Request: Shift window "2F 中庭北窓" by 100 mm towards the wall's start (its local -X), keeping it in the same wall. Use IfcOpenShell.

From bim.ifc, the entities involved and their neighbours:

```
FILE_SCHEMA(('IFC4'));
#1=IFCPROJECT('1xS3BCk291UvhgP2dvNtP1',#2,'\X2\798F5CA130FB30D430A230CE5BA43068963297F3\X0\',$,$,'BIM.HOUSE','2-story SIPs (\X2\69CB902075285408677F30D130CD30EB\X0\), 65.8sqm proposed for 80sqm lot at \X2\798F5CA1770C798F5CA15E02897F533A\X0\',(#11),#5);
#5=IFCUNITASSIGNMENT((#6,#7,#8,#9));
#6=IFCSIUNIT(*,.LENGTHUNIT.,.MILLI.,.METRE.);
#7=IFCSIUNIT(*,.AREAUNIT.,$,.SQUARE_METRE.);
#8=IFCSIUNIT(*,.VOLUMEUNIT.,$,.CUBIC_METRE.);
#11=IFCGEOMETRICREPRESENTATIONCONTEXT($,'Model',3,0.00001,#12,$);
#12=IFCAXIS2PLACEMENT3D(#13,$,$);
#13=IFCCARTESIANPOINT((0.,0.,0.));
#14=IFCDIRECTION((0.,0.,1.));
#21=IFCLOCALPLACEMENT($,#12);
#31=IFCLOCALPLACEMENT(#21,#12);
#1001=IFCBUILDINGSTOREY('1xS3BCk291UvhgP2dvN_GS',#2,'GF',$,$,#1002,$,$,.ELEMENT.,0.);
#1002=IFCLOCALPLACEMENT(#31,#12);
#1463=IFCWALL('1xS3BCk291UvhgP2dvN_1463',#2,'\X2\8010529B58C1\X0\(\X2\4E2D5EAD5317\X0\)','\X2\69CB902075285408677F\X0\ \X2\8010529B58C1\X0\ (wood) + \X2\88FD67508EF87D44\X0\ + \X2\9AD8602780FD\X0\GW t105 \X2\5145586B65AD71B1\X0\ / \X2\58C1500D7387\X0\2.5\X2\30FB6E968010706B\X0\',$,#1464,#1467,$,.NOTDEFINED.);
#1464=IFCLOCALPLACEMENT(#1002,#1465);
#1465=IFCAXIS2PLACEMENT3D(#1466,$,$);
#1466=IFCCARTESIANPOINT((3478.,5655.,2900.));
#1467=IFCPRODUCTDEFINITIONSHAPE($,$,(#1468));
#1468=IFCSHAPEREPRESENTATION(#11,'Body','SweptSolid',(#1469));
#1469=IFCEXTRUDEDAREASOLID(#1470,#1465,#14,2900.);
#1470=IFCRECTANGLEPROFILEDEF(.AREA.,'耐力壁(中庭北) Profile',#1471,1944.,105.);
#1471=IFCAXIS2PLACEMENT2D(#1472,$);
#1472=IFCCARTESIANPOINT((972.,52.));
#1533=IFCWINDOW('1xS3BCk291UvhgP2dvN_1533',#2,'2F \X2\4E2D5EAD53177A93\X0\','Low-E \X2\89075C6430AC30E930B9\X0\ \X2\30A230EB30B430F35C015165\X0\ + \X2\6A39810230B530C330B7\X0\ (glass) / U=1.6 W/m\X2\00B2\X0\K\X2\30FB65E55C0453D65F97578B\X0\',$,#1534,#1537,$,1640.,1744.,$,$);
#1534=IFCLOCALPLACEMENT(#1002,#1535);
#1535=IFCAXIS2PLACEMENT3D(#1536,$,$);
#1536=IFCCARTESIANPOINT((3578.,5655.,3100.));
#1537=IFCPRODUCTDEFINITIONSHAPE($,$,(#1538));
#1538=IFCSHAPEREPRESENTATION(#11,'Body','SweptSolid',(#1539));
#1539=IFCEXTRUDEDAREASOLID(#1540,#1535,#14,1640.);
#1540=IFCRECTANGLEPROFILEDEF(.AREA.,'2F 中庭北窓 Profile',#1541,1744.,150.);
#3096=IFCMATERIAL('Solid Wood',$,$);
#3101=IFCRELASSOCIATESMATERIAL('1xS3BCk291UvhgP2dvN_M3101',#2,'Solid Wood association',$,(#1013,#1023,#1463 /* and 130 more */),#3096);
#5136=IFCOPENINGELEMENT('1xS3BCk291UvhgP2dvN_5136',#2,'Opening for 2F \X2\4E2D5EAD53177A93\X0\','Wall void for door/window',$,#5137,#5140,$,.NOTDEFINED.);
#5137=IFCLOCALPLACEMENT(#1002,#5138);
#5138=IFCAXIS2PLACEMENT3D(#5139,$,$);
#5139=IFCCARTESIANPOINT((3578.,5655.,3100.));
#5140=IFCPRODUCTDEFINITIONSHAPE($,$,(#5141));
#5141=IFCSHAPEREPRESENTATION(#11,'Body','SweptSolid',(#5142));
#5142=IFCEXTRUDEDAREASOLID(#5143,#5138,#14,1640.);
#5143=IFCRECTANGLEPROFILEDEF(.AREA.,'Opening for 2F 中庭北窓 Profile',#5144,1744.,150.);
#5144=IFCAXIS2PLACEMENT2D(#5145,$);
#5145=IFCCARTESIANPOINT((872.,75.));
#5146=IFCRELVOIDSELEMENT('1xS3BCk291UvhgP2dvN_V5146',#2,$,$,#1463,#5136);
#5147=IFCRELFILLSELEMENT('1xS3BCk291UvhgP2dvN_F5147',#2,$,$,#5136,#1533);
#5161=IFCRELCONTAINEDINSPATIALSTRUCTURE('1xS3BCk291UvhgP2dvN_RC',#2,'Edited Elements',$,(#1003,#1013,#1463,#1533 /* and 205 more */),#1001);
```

```python
import ifcopenshell
import ifcopenshell.api.geometry
import ifcopenshell.util.placement
import ifcopenshell.util.unit

model = ifcopenshell.open("bim.ifc")
unit_scale = ifcopenshell.util.unit.calculate_unit_scale(model)

window = model.by_guid("1xS3BCk291UvhgP2dvN_1533")
opening = window.FillsVoids[0].RelatingOpeningElement
wall = opening.VoidsElements[0].RelatingBuildingElement

wall_matrix = ifcopenshell.util.placement.get_local_placement(wall.ObjectPlacement)
shift = wall_matrix[:3, 0] * -0.1 / unit_scale
before = ifcopenshell.util.placement.get_local_placement(window.ObjectPlacement)[:3, 3].copy()

# The window is not placed relative to its opening, so move both.
for product in (opening, window):
    matrix = ifcopenshell.util.placement.get_local_placement(product.ObjectPlacement)
    matrix[:3, 3] += shift
    ifcopenshell.api.geometry.edit_object_placement(model, product=product, matrix=matrix, is_si=False)

after = ifcopenshell.util.placement.get_local_placement(window.ObjectPlacement)[:3, 3]
print("window moved by", (after - before).round(3) + 0.0)

model.write("bim_rev.ifc")
```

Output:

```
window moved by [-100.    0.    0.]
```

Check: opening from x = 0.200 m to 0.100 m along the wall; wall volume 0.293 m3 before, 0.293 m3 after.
